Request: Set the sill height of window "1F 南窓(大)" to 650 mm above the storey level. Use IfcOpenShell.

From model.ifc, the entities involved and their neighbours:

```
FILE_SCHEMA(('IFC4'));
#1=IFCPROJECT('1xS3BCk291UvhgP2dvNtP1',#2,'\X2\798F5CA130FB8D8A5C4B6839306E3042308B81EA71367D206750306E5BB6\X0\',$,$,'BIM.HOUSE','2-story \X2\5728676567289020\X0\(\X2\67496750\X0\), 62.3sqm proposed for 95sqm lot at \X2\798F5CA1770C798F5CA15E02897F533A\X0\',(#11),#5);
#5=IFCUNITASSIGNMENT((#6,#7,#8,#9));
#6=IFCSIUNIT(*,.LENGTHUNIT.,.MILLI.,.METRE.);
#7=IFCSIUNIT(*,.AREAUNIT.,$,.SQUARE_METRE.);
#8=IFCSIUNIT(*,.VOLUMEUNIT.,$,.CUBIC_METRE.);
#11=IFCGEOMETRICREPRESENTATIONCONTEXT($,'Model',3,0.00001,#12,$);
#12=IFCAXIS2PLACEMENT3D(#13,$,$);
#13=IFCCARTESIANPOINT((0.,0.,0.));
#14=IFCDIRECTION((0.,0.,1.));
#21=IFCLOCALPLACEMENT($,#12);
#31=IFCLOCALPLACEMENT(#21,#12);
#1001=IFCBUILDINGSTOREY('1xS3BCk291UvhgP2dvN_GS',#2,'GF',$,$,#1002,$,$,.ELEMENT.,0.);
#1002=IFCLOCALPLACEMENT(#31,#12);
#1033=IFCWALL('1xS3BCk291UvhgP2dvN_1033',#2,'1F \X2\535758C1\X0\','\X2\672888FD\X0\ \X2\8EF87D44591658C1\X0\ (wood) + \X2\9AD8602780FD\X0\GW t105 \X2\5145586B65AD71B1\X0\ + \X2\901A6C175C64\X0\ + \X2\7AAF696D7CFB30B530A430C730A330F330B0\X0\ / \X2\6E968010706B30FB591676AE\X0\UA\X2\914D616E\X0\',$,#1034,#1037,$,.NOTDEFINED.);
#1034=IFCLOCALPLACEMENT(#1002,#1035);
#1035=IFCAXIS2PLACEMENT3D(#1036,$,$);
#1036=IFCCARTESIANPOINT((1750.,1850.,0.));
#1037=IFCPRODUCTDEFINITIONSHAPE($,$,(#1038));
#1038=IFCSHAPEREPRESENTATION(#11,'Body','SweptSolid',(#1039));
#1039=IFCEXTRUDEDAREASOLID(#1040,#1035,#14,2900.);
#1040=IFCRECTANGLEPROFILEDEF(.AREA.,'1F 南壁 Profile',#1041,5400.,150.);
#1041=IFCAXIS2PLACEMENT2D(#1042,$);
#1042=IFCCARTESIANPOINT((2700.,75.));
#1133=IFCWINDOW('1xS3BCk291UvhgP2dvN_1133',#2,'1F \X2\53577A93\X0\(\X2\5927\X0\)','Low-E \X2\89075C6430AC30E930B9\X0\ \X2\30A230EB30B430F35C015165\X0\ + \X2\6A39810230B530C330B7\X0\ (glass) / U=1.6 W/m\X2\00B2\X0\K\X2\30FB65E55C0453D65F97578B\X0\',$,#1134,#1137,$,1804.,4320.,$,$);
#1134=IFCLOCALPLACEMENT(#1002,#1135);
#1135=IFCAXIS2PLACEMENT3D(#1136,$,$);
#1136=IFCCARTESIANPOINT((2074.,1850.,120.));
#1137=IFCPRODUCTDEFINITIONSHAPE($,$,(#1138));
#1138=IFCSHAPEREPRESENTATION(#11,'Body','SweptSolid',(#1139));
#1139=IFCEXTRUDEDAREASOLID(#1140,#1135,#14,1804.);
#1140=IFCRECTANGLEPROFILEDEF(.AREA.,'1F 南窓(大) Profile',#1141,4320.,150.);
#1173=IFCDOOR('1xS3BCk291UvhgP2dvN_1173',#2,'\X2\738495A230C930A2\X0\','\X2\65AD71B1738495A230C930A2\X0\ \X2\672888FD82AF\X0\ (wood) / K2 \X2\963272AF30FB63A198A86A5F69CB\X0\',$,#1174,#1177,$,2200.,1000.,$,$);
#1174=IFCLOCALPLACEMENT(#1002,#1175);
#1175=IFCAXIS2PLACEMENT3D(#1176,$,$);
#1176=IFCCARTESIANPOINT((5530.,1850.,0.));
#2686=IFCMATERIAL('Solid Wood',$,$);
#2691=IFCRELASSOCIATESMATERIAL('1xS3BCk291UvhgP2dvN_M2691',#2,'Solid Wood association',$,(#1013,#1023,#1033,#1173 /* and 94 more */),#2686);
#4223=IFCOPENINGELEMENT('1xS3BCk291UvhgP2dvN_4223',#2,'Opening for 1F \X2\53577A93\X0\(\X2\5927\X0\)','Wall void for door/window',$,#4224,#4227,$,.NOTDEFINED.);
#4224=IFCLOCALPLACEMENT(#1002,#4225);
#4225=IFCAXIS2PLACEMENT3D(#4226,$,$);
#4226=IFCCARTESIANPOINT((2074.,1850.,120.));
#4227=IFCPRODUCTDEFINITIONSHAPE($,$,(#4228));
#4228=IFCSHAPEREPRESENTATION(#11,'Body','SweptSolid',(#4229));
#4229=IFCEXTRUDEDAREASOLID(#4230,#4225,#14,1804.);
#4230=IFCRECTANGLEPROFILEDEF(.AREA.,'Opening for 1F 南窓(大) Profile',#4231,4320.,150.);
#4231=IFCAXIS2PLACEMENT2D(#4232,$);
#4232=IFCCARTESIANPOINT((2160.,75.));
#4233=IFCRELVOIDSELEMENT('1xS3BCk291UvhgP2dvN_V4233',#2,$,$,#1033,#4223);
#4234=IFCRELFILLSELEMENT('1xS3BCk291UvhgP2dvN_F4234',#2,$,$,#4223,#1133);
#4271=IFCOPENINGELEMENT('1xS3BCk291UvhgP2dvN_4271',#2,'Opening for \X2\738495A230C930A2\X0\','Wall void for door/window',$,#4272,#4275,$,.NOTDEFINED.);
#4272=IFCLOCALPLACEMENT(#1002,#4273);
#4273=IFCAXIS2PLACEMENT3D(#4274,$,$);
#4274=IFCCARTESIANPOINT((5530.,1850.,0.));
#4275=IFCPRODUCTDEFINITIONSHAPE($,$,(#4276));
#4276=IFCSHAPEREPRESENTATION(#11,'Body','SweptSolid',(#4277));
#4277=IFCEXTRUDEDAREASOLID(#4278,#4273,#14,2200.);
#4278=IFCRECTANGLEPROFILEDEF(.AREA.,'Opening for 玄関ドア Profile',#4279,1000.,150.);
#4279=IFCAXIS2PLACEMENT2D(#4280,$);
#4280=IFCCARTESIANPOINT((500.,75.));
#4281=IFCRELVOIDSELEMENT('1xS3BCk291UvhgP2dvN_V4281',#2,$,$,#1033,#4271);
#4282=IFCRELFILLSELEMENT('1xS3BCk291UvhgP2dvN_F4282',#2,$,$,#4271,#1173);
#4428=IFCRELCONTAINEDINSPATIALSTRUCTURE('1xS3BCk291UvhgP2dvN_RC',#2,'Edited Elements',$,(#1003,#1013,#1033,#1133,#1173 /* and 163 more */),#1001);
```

```python
import numpy as np
import ifcopenshell
import ifcopenshell.api.geometry
import ifcopenshell.geom
import ifcopenshell.util.element
import ifcopenshell.util.placement
import ifcopenshell.util.shape
import ifcopenshell.util.unit

model = ifcopenshell.open("model.ifc")
unit_scale = ifcopenshell.util.unit.calculate_unit_scale(model)

window = model.by_guid("1xS3BCk291UvhgP2dvN_1133")
opening = window.FillsVoids[0].RelatingOpeningElement
storey = ifcopenshell.util.element.get_container(window, ifc_class="IfcBuildingStorey")
level = ifcopenshell.util.placement.get_local_placement(storey.ObjectPlacement)[2, 3]

# The opening's origin need not be at the sill, so measure its lowest point.
shape = ifcopenshell.geom.create_shape(ifcopenshell.geom.settings(), opening)
bottom = ifcopenshell.util.shape.get_shape_bottom_elevation(shape, shape.geometry) / unit_scale
dz = level + 650.0 - bottom

shift = np.array([0.0, 0.0, dz])
# The window is not placed relative to its opening, so move both.
for product in (opening, window):
    matrix = ifcopenshell.util.placement.get_local_placement(product.ObjectPlacement)
    matrix[:3, 3] += shift
    ifcopenshell.api.geometry.edit_object_placement(model, product=product, matrix=matrix, is_si=False)

print(f"moved by {dz * unit_scale:+.3f} m")

model.write("model_updated.ifc")
```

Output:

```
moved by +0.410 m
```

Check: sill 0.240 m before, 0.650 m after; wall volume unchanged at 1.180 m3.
